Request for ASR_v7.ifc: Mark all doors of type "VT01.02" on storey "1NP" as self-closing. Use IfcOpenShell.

First a look at what the model holds.

```python
import ifcopenshell
import ifcopenshell.util.element

model = ifcopenshell.open("ASR_v7.ifc")
print(model.schema)
storey = next(s for s in model.by_type("IfcBuildingStorey") if s.Name == "1NP")
doors = [e for e in ifcopenshell.util.element.get_decomposition(storey) if e.is_a("IfcDoor")]
seen = {}
for e in doors:
    element_type = ifcopenshell.util.element.get_type(e)
    key = (element_type.Name if element_type != e and element_type else None, ifcopenshell.util.element.get_pset(e, "Pset_DoorCommon", "SelfClosing"))
    seen[key] = seen.get(key, 0) + 1
for (name, value), count in sorted(seen.items(), key=str):
    print(count, "x", name, "|", value)
```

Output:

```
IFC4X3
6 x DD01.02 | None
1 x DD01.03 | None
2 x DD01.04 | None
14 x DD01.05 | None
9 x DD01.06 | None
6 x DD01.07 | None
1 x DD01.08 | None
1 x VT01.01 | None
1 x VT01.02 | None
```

```python
import ifcopenshell
import ifcopenshell.api.pset
import ifcopenshell.util.element

model = ifcopenshell.open("ASR_v7.ifc")

storey = next(s for s in model.by_type("IfcBuildingStorey") if s.Name == "1NP")
doors = [e for e in ifcopenshell.util.element.get_decomposition(storey) if e.is_a("IfcDoor")]

count = 0
for e in doors:
    element_type = ifcopenshell.util.element.get_type(e)
    if element_type in (None, e) or element_type.Name != "VT01.02":
        continue
    # add_pset returns the element's existing set when there is one.
    pset = ifcopenshell.api.pset.add_pset(model, product=e, name="Pset_DoorCommon")
    ifcopenshell.api.pset.edit_pset(model, pset=pset, properties={"SelfClosing": True})
    count += 1

print(count, "doors updated")

model.write("ASR_v7_edited.ifc")
```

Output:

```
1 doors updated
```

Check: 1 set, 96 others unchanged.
